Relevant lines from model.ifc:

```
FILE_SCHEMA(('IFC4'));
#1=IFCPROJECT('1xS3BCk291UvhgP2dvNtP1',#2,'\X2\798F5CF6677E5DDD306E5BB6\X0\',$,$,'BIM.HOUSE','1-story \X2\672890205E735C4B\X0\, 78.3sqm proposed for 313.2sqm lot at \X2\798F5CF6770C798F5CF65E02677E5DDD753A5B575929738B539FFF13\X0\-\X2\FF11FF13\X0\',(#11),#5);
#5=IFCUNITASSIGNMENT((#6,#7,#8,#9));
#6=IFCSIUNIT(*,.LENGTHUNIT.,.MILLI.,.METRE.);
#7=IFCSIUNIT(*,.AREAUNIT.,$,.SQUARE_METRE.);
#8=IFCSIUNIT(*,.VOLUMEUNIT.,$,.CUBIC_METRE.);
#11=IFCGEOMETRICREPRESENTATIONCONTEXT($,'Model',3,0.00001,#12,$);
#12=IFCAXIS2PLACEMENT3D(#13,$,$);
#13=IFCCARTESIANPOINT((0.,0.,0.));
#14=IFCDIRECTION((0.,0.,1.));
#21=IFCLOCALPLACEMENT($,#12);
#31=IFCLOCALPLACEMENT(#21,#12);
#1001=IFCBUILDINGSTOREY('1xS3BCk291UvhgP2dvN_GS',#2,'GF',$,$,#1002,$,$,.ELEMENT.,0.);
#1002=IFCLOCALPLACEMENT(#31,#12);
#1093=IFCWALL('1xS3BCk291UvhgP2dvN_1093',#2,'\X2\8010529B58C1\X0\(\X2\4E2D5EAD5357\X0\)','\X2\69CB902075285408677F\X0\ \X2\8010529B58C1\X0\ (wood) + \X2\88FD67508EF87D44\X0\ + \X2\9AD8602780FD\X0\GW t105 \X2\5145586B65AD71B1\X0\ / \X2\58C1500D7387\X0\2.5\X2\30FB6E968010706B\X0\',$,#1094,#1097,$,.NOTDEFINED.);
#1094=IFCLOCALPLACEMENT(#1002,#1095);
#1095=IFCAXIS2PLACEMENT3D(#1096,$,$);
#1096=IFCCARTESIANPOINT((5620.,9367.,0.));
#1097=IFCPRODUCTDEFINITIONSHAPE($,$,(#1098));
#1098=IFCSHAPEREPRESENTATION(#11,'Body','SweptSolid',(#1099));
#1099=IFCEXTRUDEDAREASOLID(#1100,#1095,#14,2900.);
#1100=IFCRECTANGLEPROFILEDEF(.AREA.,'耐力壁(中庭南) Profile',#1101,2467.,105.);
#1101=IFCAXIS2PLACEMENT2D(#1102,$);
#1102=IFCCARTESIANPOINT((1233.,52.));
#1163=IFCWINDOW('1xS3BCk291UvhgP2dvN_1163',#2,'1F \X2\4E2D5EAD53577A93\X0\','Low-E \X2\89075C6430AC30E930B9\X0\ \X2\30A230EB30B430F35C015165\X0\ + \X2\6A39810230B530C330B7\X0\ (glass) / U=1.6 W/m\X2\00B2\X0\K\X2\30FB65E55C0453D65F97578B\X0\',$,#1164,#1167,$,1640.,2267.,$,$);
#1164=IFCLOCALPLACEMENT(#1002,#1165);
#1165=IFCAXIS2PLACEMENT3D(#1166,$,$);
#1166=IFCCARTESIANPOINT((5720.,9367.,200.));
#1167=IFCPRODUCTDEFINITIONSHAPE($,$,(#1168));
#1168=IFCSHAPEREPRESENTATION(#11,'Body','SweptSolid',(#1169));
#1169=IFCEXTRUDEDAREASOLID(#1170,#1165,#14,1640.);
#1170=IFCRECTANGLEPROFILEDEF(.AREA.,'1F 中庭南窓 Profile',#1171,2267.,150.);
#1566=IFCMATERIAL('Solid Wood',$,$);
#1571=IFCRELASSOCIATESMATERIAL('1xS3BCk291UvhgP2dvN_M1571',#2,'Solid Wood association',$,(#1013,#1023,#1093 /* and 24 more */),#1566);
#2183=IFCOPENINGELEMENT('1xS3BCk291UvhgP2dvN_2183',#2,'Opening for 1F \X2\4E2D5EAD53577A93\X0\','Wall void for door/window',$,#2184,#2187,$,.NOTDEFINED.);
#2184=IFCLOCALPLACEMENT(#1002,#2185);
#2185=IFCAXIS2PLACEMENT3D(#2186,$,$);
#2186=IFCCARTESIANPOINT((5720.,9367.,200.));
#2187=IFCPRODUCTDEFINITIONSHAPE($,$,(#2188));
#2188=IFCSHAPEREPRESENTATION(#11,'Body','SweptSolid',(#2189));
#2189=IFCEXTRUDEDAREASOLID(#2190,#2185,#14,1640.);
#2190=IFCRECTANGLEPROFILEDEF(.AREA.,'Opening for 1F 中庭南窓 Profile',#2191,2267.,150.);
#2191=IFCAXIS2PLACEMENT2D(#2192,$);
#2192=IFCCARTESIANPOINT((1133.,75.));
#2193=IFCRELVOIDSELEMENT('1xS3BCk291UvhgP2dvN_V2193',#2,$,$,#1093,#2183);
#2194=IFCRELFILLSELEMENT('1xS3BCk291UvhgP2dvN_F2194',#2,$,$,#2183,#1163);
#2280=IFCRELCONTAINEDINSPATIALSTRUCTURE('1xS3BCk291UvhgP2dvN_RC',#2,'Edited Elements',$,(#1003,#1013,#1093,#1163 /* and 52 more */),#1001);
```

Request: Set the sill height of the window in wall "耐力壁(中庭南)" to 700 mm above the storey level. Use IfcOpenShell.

```python
import numpy as np
import ifcopenshell
import ifcopenshell.api.geometry
import ifcopenshell.geom
import ifcopenshell.util.element
import ifcopenshell.util.placement
import ifcopenshell.util.shape
import ifcopenshell.util.unit

model = ifcopenshell.open("model.ifc")
unit_scale = ifcopenshell.util.unit.calculate_unit_scale(model)

window = model.by_guid("1xS3BCk291UvhgP2dvN_1163")
opening = window.FillsVoids[0].RelatingOpeningElement
storey = ifcopenshell.util.element.get_container(window, ifc_class="IfcBuildingStorey")
level = ifcopenshell.util.placement.get_local_placement(storey.ObjectPlacement)[2, 3]

# The opening's origin need not be at the sill, so measure its lowest point.
shape = ifcopenshell.geom.create_shape(ifcopenshell.geom.settings(), opening)
bottom = ifcopenshell.util.shape.get_shape_bottom_elevation(shape, shape.geometry) / unit_scale
dz = level + 700.0 - bottom

shift = np.array([0.0, 0.0, dz])
# The window is not placed relative to its opening, so move both.
for product in (opening, window):
    matrix = ifcopenshell.util.placement.get_local_placement(product.ObjectPlacement)
    matrix[:3, 3] += shift
    ifcopenshell.api.geometry.edit_object_placement(model, product=product, matrix=matrix, is_si=False)

print(f"moved by {dz * unit_scale:+.3f} m")

model.write("model_updated.ifc")
```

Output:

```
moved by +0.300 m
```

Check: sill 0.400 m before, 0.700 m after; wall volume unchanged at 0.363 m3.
